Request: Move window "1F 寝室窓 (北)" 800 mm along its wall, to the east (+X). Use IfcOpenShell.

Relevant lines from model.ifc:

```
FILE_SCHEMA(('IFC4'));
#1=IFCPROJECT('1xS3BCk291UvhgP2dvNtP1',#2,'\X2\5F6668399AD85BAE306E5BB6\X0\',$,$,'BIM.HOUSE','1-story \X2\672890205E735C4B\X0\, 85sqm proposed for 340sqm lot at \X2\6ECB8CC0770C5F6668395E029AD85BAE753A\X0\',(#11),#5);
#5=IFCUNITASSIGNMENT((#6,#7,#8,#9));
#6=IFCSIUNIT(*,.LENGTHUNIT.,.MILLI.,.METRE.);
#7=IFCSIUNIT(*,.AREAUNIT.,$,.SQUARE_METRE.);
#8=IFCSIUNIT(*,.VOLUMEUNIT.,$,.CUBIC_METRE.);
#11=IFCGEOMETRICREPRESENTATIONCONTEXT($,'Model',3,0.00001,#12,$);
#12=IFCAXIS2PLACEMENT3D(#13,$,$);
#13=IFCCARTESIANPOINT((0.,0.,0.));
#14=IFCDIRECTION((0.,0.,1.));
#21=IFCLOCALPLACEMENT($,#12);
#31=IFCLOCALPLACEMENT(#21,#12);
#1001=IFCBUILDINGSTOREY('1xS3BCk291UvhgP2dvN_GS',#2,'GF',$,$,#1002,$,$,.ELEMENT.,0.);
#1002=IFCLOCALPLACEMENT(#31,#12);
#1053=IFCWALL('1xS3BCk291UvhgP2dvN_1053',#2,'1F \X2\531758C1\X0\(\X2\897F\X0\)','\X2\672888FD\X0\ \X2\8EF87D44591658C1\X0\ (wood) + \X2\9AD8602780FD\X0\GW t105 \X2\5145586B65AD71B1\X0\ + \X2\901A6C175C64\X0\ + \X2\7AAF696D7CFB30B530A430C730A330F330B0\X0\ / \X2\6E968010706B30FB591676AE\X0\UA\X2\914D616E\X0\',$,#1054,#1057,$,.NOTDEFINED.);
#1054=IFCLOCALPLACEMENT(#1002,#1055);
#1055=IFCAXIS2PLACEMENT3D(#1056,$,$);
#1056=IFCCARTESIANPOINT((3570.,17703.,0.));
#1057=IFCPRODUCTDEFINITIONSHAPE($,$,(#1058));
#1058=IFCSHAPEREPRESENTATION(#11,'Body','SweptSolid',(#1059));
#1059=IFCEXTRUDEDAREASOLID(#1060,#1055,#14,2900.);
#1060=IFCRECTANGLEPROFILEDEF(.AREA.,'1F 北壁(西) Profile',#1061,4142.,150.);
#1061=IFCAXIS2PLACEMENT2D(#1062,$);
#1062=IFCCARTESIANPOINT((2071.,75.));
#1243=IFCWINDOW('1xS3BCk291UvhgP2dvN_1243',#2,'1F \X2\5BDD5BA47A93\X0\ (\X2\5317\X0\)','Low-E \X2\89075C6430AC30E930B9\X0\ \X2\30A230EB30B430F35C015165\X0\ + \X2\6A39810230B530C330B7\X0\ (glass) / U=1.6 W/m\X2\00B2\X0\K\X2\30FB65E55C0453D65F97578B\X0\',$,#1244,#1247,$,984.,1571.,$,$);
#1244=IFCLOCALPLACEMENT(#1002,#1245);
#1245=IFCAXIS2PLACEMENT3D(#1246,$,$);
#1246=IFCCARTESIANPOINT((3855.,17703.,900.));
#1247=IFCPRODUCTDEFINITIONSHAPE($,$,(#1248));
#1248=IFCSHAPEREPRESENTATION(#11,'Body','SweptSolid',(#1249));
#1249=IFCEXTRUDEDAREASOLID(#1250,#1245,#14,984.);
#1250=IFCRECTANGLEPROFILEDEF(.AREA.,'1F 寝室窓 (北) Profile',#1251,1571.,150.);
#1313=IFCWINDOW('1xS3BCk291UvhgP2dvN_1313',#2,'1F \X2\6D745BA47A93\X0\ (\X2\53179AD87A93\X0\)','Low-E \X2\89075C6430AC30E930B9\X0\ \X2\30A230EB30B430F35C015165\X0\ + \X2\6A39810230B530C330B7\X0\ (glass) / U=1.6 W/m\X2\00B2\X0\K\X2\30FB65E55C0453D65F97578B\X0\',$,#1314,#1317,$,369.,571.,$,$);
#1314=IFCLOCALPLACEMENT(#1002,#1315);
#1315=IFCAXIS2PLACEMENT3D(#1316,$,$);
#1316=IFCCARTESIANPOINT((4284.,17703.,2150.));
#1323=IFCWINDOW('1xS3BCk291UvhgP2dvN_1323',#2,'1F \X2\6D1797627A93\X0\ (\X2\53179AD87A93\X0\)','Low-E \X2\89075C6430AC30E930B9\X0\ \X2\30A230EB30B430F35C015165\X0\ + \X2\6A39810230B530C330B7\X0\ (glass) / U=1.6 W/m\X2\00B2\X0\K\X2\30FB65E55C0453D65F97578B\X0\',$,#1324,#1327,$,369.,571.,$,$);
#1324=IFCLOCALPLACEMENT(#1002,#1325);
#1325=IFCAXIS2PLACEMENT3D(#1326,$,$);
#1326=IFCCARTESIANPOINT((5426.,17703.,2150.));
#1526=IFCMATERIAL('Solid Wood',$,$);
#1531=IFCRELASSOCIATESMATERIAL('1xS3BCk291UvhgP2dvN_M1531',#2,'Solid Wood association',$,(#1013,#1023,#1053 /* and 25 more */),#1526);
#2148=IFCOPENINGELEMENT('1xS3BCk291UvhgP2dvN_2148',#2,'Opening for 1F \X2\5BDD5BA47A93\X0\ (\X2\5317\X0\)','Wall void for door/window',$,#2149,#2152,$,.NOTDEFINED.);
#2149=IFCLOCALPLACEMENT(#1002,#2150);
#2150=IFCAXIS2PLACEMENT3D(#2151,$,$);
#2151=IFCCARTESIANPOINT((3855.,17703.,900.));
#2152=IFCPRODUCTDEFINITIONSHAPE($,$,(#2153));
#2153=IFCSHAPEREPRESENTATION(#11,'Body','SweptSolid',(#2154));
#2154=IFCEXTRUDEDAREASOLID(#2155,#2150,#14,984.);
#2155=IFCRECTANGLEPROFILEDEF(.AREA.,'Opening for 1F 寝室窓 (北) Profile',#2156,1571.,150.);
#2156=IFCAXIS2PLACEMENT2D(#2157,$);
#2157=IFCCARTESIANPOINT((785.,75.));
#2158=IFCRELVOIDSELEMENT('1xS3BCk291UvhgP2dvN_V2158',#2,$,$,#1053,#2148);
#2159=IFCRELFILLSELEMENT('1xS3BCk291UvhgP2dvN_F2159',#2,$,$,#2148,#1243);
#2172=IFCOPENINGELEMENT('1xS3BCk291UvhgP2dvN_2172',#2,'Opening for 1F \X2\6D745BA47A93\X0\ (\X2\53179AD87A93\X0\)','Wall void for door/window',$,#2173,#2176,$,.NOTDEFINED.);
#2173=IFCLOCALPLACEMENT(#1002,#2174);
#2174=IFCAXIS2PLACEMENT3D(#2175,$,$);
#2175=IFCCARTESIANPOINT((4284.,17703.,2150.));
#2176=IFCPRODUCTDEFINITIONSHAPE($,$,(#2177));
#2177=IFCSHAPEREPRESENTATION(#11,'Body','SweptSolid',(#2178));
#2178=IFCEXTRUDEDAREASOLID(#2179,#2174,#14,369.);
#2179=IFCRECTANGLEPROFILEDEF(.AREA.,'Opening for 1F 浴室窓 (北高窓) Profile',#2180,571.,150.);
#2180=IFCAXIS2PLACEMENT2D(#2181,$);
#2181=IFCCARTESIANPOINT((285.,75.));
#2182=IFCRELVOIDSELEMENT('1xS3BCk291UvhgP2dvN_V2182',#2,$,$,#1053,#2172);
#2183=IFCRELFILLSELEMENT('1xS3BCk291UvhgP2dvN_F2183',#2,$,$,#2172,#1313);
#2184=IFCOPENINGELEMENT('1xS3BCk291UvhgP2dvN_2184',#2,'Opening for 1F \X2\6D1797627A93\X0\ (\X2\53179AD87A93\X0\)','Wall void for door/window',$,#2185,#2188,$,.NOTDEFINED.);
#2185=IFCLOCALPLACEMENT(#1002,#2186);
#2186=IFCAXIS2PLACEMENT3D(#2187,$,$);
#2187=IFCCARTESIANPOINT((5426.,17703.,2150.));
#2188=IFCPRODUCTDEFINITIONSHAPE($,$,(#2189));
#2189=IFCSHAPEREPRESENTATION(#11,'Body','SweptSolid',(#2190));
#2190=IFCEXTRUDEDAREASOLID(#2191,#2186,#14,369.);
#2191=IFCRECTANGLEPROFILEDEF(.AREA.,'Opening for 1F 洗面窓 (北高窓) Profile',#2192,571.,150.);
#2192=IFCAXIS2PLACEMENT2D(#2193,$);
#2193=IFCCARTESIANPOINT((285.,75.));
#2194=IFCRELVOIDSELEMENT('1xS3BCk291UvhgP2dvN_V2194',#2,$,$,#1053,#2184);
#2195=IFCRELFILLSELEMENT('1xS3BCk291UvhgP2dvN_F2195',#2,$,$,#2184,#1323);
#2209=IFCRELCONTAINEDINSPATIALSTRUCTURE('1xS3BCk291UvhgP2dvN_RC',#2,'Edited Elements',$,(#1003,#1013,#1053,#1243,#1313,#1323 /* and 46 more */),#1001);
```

```python
import ifcopenshell
import ifcopenshell.api.geometry
import ifcopenshell.util.placement
import ifcopenshell.util.unit

model = ifcopenshell.open("model.ifc")
unit_scale = ifcopenshell.util.unit.calculate_unit_scale(model)

window = model.by_guid("1xS3BCk291UvhgP2dvN_1243")
opening = window.FillsVoids[0].RelatingOpeningElement
wall = opening.VoidsElements[0].RelatingBuildingElement

wall_matrix = ifcopenshell.util.placement.get_local_placement(wall.ObjectPlacement)
shift = wall_matrix[:3, 0] * 0.8 / unit_scale
before = ifcopenshell.util.placement.get_local_placement(window.ObjectPlacement)[:3, 3].copy()

# The window is not placed relative to its opening, so move both.
for product in (opening, window):
    matrix = ifcopenshell.util.placement.get_local_placement(product.ObjectPlacement)
    matrix[:3, 3] += shift
    ifcopenshell.api.geometry.edit_object_placement(model, product=product, matrix=matrix, is_si=False)

after = ifcopenshell.util.placement.get_local_placement(window.ObjectPlacement)[:3, 3]
print("window moved by", (after - before).round(3) + 0.0)

model.write("model_updated.ifc")
```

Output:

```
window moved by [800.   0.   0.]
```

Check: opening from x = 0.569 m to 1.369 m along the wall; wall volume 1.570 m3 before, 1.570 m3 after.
